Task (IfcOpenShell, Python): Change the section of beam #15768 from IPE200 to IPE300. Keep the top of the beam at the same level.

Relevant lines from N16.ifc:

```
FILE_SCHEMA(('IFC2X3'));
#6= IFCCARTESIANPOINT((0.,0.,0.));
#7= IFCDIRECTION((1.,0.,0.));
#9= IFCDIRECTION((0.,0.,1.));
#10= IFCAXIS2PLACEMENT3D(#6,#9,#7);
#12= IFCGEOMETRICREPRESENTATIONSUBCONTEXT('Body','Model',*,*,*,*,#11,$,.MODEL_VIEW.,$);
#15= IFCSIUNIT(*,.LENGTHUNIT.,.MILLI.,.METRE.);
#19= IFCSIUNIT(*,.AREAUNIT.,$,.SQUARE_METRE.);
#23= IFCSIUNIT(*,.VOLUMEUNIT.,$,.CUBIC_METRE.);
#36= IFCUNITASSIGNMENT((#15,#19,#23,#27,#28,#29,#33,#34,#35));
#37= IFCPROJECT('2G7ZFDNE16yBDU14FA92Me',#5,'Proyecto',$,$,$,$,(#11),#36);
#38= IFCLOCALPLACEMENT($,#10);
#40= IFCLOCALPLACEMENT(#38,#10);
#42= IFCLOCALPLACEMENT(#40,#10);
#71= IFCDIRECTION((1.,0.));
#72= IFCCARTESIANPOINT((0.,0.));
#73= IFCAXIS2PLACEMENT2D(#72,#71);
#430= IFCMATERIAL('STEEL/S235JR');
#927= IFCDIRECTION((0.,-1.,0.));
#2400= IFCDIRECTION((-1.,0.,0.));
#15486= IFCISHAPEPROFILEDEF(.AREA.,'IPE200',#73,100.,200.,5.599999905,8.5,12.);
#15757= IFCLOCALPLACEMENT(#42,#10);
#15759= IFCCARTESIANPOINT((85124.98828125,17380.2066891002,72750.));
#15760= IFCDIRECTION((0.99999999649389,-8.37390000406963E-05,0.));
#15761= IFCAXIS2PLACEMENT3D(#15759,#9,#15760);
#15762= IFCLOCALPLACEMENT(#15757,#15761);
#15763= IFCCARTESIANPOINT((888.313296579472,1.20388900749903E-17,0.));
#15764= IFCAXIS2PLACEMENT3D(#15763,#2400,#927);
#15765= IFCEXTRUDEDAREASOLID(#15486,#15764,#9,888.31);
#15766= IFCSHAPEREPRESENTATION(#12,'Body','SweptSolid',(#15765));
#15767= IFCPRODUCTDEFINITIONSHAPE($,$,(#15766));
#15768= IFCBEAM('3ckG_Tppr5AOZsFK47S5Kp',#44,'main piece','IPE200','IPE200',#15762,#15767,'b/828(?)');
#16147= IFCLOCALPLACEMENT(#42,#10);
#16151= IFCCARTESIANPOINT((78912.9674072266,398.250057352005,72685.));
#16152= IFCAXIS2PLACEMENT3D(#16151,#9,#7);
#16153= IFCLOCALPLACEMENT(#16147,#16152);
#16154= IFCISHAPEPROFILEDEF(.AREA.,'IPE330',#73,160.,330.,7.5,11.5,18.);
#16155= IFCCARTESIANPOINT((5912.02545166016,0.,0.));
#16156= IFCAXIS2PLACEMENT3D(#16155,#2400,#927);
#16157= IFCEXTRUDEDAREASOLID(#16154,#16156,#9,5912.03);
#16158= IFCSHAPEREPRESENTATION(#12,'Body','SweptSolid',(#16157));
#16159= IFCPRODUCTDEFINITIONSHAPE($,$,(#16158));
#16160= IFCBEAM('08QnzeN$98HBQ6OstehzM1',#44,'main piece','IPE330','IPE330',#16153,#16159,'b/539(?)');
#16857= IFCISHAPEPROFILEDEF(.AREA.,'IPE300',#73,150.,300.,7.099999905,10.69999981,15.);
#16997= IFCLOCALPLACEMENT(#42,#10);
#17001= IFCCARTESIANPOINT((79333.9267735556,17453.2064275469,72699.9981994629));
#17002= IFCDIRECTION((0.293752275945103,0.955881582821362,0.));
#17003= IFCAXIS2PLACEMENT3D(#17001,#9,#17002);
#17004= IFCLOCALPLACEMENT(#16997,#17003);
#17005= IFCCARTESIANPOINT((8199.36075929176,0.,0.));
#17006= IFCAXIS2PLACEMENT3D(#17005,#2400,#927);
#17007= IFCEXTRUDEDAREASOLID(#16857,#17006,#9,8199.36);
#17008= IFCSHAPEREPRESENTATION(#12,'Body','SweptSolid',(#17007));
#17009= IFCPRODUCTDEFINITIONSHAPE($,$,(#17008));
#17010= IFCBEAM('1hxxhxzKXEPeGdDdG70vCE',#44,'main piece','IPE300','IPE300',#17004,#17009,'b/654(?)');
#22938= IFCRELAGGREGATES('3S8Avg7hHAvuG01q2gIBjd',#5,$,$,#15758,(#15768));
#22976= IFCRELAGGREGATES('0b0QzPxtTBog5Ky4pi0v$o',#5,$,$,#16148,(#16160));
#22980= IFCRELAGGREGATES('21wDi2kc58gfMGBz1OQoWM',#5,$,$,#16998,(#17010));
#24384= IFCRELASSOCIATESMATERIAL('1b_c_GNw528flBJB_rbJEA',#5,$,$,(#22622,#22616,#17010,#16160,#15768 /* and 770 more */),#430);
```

```python
import ifcopenshell
import ifcopenshell.util.element
import ifcopenshell.util.representation

model = ifcopenshell.open("N16.ifc")

member = model.by_id(15768)
source = next(p for p in model.by_type("IfcIShapeProfileDef") if p.ProfileName == "IPE300")

body = ifcopenshell.util.representation.get_representation(member, "Model", "Body")
solid = body.Items[0]
old_profile = solid.SweptArea

# Copy the section's sizes but keep this member's own profile position.
profile = ifcopenshell.util.element.copy(model, source)
# Profiles are centred, so shift by half the change in depth to hold the top.
shift = (old_profile.OverallDepth - profile.OverallDepth) / 2
x, y = old_profile.Position.Location.Coordinates
up = (0.0, 1.0)  # upwards, in the solid's own plane
location = model.createIfcCartesianPoint((x + up[0] * shift, y + up[1] * shift))
profile.Position = model.createIfcAxis2Placement2D(location, old_profile.Position.RefDirection)
solid.SweptArea = profile
if not model.get_total_inverses(old_profile):
    ifcopenshell.util.element.remove_deep2(model, old_profile)
member.Description = member.Description.replace("IPE200", "IPE300")
member.ObjectType = member.ObjectType.replace("IPE200", "IPE300")

print(solid.SweptArea)

model.write("N16_edited.ifc")
```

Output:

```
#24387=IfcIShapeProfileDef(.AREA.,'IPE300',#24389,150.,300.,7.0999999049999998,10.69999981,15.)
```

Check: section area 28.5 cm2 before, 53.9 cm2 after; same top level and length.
